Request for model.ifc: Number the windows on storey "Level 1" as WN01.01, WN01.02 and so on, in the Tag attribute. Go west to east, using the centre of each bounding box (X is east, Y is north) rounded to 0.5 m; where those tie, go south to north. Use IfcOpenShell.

First a look at what the model holds.

```python
import ifcopenshell
import ifcopenshell.util.element
import ifcopenshell.util.placement

model = ifcopenshell.open("model.ifc")
print(model.schema)
storey = next(s for s in model.by_type("IfcBuildingStorey") if s.Name == "Level 1")
windows = [e for e in ifcopenshell.util.element.get_decomposition(storey) if e.is_a("IfcWindow")]
for e in sorted(windows, key=lambda e: e.id()):
    origin = ifcopenshell.util.placement.get_local_placement(e.ObjectPlacement)[:3, 3]
    print(e.id(), e.Tag, e.Name, origin.round(2) + 0.0, sep=" | ")
```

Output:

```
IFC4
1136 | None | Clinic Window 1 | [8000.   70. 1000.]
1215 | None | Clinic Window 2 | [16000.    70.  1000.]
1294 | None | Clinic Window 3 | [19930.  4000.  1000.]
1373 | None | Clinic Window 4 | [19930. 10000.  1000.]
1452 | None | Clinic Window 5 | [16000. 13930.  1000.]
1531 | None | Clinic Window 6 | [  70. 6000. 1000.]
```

```python
import ifcopenshell
import ifcopenshell.geom
import ifcopenshell.util.element
import ifcopenshell.util.shape

model = ifcopenshell.open("model.ifc")
settings = ifcopenshell.geom.settings()
settings.set("use-world-coords", True)


def centre(element):
    shape = ifcopenshell.geom.create_shape(settings, element)
    return ifcopenshell.util.shape.get_bbox_centroid(shape.geometry)


storey = next(s for s in model.by_type("IfcBuildingStorey") if s.Name == "Level 1")
windows = [e for e in ifcopenshell.util.element.get_decomposition(storey) if e.is_a("IfcWindow")]

# Insertion points can sit at a corner or the storey origin, so sort by the geometry (in metres).
centres = {e: centre(e) for e in windows}
windows.sort(key=lambda e: (round(centres[e][0] / 0.5), centres[e][1]))

for i, e in enumerate(windows, start=1):
    number = f"WN01.{i:02d}"
    e.Tag = number
    print(e.id(), number)

model.write("model_rev.ifc")
```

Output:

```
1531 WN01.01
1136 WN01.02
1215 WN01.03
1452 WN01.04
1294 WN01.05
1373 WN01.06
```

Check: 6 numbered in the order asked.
